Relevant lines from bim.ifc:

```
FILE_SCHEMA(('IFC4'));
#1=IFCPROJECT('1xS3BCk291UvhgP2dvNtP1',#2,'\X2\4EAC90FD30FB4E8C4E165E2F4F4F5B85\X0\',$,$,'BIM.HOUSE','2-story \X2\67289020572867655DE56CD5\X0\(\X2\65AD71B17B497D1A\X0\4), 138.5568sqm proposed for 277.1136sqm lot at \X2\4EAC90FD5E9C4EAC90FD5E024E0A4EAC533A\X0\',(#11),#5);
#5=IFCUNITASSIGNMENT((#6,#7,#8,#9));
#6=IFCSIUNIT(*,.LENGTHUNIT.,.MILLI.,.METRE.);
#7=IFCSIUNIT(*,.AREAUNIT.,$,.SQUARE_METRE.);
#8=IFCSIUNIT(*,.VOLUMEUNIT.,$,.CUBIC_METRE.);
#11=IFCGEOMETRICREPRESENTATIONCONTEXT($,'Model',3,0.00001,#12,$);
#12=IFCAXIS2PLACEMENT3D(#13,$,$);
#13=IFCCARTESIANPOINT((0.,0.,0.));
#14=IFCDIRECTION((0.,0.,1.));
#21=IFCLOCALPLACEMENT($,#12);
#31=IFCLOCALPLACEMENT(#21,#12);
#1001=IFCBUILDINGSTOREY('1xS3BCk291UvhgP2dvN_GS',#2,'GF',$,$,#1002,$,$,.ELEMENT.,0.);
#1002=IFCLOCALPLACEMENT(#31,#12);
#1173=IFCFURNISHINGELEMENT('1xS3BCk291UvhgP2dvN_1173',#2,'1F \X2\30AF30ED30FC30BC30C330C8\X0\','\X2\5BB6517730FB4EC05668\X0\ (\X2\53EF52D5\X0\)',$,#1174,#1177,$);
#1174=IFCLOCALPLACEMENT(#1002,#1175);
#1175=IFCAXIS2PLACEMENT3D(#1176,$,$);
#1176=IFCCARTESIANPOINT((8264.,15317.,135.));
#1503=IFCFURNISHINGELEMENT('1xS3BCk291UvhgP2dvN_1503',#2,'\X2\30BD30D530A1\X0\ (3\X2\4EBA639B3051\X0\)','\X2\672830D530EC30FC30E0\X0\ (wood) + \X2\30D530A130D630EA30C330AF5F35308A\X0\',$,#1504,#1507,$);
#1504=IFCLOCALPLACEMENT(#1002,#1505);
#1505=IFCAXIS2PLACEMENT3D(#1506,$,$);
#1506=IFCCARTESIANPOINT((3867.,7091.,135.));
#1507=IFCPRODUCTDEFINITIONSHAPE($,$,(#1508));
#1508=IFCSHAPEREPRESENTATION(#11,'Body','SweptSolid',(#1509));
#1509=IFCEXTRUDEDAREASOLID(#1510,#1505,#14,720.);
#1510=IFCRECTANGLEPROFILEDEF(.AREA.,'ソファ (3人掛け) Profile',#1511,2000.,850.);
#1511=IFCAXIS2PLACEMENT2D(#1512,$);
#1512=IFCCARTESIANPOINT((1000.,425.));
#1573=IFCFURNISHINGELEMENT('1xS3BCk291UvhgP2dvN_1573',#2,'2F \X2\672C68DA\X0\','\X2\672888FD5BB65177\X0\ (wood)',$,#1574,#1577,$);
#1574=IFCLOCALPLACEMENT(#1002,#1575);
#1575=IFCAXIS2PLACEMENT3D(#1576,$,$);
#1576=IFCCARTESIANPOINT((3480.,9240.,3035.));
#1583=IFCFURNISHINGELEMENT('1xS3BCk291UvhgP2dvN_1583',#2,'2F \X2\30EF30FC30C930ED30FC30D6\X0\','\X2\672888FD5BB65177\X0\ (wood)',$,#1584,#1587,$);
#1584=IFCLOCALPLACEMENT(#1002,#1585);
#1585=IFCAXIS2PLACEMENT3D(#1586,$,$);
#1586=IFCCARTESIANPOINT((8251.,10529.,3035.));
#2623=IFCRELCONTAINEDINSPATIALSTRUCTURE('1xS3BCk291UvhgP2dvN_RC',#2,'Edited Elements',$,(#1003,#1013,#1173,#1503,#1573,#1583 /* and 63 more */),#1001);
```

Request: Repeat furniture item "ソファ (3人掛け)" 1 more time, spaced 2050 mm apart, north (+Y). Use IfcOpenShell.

```python
import numpy as np
import ifcopenshell
import ifcopenshell.api.geometry
import ifcopenshell.api.root
import ifcopenshell.util.element
import ifcopenshell.util.placement

model = ifcopenshell.open("bim.ifc")


def reuse_history(source, copy):
    """copy_class also copies each property set's owner history, people and application; keep the originals."""
    for rel in copy.IsDefinedBy:
        if rel.is_a("IfcRelDefinesByProperties") and (history := rel.RelatingPropertyDefinition.OwnerHistory):
            rel.RelatingPropertyDefinition.OwnerHistory = source.OwnerHistory
            ifcopenshell.util.element.remove_deep2(model, history)


source = model.by_id(1503)
base = ifcopenshell.util.placement.get_local_placement(source.ObjectPlacement)
step = np.array([0.0, 1.0, 0.0]) * 2050.0

for i in range(1, 2):
    copy = ifcopenshell.api.root.copy_class(model, product=source)
    copy.Representation = ifcopenshell.util.element.copy_deep(
        model, source.Representation, exclude=["IfcGeometricRepresentationContext", "IfcRepresentationMap"]
    )
    reuse_history(source, copy)
    matrix = base.copy()
    matrix[:3, 3] += i * step
    print("added at", matrix[:3, 3].round(3) + 0.0)
    ifcopenshell.api.geometry.edit_object_placement(model, product=copy, matrix=matrix, is_si=False)

model.write("bim_updated.ifc")
```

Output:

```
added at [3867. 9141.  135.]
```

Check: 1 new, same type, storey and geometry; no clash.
